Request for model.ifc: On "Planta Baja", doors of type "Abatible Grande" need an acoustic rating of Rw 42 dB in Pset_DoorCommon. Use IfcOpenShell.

First a look at what the model holds.

```python
import ifcopenshell
import ifcopenshell.util.element

model = ifcopenshell.open("model.ifc")
print(model.schema)
storey = next(s for s in model.by_type("IfcBuildingStorey") if s.Name == "Planta Baja")
doors = [e for e in ifcopenshell.util.element.get_decomposition(storey) if e.is_a("IfcDoor")]
seen = {}
for e in doors:
    element_type = ifcopenshell.util.element.get_type(e)
    key = (element_type.Name if element_type != e and element_type else None, ifcopenshell.util.element.get_pset(e, "Pset_DoorCommon", "AcousticRating"))
    seen[key] = seen.get(key, 0) + 1
for (name, value), count in sorted(seen.items(), key=str):
    print(count, "x", name, "|", value)
```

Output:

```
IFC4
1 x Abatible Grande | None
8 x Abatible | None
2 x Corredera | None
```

```python
import ifcopenshell
import ifcopenshell.api.pset
import ifcopenshell.util.element

model = ifcopenshell.open("model.ifc")

storey = next(s for s in model.by_type("IfcBuildingStorey") if s.Name == "Planta Baja")
doors = [e for e in ifcopenshell.util.element.get_decomposition(storey) if e.is_a("IfcDoor")]

count = 0
for e in doors:
    element_type = ifcopenshell.util.element.get_type(e)
    if element_type in (None, e) or element_type.Name != "Abatible Grande":
        continue
    # add_pset returns the element's existing set when there is one.
    pset = ifcopenshell.api.pset.add_pset(model, product=e, name="Pset_DoorCommon")
    ifcopenshell.api.pset.edit_pset(model, pset=pset, properties={"AcousticRating": "Rw 42 dB"})
    count += 1

print(count, "doors updated")

model.write("model_v2.ifc")
```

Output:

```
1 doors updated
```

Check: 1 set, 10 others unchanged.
